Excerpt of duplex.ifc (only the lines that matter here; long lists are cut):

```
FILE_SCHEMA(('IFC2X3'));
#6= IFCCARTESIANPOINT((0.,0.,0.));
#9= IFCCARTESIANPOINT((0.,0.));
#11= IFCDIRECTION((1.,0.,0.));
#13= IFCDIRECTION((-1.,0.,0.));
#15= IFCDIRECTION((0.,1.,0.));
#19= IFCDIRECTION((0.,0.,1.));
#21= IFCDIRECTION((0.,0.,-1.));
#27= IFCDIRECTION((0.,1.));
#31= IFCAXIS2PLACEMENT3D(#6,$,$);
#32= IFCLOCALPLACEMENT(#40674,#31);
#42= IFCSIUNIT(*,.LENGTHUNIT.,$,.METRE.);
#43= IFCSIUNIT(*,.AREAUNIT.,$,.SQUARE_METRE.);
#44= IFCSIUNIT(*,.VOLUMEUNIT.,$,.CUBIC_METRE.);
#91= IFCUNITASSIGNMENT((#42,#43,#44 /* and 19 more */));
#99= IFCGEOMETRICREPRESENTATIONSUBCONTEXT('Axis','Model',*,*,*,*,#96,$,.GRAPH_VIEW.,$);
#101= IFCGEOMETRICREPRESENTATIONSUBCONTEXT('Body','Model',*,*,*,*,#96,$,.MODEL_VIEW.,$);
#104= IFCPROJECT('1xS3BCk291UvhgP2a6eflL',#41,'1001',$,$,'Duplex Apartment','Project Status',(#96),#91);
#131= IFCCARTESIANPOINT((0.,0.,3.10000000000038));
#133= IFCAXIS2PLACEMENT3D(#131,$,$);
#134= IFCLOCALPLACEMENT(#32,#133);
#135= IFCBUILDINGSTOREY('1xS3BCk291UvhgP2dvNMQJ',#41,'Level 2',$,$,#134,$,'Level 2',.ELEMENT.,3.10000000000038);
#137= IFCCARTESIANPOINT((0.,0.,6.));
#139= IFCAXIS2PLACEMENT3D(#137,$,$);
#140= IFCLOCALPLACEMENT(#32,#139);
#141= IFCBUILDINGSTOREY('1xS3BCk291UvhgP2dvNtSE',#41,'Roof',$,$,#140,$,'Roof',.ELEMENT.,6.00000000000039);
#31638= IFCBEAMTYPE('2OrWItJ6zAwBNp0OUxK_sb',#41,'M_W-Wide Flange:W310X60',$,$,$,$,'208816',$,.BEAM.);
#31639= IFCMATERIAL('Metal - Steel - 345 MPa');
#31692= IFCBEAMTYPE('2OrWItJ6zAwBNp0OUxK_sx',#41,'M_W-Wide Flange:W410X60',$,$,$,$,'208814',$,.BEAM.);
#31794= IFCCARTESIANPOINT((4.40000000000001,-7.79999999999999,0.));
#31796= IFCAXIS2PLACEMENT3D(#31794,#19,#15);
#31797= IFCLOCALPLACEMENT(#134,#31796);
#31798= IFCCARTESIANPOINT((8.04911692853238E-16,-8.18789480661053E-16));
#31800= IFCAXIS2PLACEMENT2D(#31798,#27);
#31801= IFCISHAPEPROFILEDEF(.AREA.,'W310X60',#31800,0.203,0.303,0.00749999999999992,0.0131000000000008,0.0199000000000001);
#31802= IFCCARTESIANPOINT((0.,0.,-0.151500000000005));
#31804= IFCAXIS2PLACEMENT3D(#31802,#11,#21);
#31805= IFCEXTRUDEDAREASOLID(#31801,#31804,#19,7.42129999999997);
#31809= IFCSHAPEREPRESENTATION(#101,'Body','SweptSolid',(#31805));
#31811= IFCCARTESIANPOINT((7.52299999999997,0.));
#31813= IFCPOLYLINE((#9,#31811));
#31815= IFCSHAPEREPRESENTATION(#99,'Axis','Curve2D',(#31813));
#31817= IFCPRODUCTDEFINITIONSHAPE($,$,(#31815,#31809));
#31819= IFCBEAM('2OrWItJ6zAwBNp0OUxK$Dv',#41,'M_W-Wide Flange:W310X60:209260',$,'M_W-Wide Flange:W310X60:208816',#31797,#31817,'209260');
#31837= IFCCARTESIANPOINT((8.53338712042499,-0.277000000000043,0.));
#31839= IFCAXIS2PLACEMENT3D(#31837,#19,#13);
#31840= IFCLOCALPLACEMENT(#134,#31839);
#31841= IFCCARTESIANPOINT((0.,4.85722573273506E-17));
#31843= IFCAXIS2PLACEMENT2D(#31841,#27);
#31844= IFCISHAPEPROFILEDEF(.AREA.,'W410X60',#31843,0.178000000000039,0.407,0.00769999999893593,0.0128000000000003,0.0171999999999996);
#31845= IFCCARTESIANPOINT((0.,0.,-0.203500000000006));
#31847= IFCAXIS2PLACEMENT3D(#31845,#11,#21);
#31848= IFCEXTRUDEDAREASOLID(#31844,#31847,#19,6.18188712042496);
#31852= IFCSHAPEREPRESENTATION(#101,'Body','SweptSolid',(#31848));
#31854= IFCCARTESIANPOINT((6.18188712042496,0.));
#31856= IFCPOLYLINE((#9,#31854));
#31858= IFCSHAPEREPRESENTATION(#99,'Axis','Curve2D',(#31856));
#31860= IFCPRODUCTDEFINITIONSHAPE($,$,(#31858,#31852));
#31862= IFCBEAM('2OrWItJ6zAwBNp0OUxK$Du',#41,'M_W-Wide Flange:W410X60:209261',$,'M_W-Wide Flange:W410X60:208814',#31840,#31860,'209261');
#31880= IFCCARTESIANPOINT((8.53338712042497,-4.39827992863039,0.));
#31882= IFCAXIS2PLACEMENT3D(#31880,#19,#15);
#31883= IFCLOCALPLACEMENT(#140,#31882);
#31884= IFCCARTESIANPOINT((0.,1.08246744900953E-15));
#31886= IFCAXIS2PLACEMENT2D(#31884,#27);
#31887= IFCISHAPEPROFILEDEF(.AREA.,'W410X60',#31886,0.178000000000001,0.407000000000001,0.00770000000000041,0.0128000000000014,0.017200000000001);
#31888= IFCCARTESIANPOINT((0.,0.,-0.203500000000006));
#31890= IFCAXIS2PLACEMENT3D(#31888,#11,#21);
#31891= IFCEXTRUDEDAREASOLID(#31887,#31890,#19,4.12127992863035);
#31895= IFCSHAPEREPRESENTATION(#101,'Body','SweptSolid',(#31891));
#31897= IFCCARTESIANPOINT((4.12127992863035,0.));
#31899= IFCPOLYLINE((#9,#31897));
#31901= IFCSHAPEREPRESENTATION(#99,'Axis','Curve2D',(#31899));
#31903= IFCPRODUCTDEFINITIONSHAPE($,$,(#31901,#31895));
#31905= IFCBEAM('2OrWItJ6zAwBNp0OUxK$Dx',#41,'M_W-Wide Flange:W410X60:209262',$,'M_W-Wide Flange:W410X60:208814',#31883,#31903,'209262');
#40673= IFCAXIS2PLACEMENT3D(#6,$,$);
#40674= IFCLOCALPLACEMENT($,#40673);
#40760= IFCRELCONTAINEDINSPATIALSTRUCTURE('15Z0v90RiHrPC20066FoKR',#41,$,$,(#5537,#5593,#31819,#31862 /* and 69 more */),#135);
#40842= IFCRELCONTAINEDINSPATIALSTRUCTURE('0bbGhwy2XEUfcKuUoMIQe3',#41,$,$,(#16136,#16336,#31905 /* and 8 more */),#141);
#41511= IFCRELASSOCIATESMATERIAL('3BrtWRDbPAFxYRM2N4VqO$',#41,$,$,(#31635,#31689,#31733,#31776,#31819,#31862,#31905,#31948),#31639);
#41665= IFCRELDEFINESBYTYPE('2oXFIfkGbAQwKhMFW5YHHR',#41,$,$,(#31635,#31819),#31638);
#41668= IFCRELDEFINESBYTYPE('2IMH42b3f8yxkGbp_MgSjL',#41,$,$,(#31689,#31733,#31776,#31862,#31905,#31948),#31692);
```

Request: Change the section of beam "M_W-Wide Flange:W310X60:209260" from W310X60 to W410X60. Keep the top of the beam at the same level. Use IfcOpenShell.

```python
import ifcopenshell
import ifcopenshell.api.type
import ifcopenshell.util.element
import ifcopenshell.util.representation

model = ifcopenshell.open("duplex.ifc")

member = model.by_id(31819)
source = next(p for p in model.by_type("IfcIShapeProfileDef") if p.ProfileName == "W410X60")

body = ifcopenshell.util.representation.get_representation(member, "Model", "Body")
solid = body.Items[0]
old_profile = solid.SweptArea

# Copy the section's sizes but keep this member's own profile position.
profile = ifcopenshell.util.element.copy(model, source)
# Profiles are centred, so shift by half the change in depth to hold the top.
shift = (old_profile.OverallDepth - profile.OverallDepth) / 2
x, y = old_profile.Position.Location.Coordinates
up = (-1.0, 0.0)  # upwards, in the solid's own plane
location = model.createIfcCartesianPoint((x + up[0] * shift, y + up[1] * shift))
profile.Position = model.createIfcAxis2Placement2D(location, old_profile.Position.RefDirection)
solid.SweptArea = profile
if not model.get_total_inverses(old_profile):
    ifcopenshell.util.element.remove_deep2(model, old_profile)

new_type = model.by_guid("2OrWItJ6zAwBNp0OUxK_sx")
ifcopenshell.api.type.assign_type(
    model, related_objects=[member], relating_type=new_type, should_map_representations=False
)
member.Name = member.Name.replace("W310X60", "W410X60")
member.ObjectType = "M_W-Wide Flange:W410X60:208816"

print(solid.SweptArea)

model.write("duplex_edited.ifc")
```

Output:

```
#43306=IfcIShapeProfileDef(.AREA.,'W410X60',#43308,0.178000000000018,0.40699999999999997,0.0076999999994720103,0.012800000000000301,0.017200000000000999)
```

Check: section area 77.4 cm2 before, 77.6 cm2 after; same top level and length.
